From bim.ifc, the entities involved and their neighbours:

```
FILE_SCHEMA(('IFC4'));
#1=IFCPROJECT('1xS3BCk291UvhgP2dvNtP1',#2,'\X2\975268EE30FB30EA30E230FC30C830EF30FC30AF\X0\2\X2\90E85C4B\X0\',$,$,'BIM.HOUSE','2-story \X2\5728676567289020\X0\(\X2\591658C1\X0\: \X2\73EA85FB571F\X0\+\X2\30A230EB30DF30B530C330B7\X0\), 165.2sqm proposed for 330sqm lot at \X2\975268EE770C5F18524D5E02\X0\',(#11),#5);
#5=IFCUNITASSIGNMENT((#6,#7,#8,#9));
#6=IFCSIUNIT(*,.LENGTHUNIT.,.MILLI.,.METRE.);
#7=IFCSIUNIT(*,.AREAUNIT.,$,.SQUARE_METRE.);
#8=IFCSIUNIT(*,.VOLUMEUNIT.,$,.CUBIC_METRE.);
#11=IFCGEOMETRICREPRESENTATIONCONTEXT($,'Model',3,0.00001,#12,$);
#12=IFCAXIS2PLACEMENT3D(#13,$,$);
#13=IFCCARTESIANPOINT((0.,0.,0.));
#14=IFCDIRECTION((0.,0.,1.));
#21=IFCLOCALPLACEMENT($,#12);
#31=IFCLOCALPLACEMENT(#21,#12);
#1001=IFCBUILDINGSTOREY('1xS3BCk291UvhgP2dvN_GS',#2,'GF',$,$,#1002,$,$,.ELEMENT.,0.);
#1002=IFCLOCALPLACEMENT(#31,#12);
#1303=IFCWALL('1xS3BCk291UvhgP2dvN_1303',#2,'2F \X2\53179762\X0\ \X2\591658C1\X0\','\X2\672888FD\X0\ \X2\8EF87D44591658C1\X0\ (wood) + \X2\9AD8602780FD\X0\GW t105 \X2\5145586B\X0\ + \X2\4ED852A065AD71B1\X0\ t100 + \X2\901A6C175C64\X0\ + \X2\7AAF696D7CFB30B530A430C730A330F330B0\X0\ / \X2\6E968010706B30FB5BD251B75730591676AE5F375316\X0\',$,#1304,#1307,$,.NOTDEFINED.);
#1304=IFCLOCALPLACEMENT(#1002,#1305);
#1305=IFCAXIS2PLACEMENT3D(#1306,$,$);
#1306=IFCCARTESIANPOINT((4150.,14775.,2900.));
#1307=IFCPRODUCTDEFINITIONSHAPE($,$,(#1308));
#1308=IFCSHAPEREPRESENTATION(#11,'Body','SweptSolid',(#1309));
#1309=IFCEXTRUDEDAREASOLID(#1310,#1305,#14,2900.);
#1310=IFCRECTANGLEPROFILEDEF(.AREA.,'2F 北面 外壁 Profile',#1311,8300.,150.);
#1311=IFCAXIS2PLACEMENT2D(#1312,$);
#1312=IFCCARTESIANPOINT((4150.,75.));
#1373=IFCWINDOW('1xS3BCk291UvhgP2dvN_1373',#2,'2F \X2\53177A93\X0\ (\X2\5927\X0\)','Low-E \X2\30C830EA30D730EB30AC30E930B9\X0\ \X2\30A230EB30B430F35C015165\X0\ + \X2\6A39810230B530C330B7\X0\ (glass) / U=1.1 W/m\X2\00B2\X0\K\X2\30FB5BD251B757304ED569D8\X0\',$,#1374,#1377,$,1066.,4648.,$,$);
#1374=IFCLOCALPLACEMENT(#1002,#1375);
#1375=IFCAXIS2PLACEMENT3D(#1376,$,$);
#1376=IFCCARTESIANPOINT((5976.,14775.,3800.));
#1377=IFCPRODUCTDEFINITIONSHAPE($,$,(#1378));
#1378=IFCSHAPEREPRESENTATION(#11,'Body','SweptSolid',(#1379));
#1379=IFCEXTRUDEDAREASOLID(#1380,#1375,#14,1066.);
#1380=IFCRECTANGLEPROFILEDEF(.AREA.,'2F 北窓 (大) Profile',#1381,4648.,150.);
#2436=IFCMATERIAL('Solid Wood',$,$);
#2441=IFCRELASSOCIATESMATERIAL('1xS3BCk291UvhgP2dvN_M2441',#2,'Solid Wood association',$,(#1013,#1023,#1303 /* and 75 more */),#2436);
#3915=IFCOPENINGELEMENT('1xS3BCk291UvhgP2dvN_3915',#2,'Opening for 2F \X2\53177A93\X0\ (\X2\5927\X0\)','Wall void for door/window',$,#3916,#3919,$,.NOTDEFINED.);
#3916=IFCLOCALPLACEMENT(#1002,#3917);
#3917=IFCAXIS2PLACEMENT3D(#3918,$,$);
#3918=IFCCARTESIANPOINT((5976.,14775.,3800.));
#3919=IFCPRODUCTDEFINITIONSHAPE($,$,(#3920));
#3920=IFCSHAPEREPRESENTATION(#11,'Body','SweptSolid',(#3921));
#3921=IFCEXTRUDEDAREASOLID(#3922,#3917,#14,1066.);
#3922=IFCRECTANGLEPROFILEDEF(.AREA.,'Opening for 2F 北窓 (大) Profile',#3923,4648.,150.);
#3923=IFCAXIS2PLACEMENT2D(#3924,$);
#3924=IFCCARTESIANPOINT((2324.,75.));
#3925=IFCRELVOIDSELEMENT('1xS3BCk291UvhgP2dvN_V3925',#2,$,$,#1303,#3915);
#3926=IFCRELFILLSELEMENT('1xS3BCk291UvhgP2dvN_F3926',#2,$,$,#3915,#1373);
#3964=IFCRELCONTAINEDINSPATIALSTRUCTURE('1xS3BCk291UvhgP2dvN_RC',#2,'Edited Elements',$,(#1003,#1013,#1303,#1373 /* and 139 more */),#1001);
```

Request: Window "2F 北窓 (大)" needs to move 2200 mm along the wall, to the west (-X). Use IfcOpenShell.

```python
import ifcopenshell
import ifcopenshell.api.geometry
import ifcopenshell.util.placement

model = ifcopenshell.open("bim.ifc")

window = model.by_id(1373)
opening = window.FillsVoids[0].RelatingOpeningElement
wall = opening.VoidsElements[0].RelatingBuildingElement

wall_matrix = ifcopenshell.util.placement.get_local_placement(wall.ObjectPlacement)
shift = wall_matrix[:3, 0] * -2200.0
before = ifcopenshell.util.placement.get_local_placement(window.ObjectPlacement)[:3, 3].copy()

# The window is not placed relative to its opening, so move both.
for product in (opening, window):
    matrix = ifcopenshell.util.placement.get_local_placement(product.ObjectPlacement)
    matrix[:3, 3] += shift
    ifcopenshell.api.geometry.edit_object_placement(model, product=product, matrix=matrix, is_si=False)

after = ifcopenshell.util.placement.get_local_placement(window.ObjectPlacement)[:3, 3]
print("window moved by", (after - before).round(3) + 0.0)

model.write("bim_v2.ifc")
```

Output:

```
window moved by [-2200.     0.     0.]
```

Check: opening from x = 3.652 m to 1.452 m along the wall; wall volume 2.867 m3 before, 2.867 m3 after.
